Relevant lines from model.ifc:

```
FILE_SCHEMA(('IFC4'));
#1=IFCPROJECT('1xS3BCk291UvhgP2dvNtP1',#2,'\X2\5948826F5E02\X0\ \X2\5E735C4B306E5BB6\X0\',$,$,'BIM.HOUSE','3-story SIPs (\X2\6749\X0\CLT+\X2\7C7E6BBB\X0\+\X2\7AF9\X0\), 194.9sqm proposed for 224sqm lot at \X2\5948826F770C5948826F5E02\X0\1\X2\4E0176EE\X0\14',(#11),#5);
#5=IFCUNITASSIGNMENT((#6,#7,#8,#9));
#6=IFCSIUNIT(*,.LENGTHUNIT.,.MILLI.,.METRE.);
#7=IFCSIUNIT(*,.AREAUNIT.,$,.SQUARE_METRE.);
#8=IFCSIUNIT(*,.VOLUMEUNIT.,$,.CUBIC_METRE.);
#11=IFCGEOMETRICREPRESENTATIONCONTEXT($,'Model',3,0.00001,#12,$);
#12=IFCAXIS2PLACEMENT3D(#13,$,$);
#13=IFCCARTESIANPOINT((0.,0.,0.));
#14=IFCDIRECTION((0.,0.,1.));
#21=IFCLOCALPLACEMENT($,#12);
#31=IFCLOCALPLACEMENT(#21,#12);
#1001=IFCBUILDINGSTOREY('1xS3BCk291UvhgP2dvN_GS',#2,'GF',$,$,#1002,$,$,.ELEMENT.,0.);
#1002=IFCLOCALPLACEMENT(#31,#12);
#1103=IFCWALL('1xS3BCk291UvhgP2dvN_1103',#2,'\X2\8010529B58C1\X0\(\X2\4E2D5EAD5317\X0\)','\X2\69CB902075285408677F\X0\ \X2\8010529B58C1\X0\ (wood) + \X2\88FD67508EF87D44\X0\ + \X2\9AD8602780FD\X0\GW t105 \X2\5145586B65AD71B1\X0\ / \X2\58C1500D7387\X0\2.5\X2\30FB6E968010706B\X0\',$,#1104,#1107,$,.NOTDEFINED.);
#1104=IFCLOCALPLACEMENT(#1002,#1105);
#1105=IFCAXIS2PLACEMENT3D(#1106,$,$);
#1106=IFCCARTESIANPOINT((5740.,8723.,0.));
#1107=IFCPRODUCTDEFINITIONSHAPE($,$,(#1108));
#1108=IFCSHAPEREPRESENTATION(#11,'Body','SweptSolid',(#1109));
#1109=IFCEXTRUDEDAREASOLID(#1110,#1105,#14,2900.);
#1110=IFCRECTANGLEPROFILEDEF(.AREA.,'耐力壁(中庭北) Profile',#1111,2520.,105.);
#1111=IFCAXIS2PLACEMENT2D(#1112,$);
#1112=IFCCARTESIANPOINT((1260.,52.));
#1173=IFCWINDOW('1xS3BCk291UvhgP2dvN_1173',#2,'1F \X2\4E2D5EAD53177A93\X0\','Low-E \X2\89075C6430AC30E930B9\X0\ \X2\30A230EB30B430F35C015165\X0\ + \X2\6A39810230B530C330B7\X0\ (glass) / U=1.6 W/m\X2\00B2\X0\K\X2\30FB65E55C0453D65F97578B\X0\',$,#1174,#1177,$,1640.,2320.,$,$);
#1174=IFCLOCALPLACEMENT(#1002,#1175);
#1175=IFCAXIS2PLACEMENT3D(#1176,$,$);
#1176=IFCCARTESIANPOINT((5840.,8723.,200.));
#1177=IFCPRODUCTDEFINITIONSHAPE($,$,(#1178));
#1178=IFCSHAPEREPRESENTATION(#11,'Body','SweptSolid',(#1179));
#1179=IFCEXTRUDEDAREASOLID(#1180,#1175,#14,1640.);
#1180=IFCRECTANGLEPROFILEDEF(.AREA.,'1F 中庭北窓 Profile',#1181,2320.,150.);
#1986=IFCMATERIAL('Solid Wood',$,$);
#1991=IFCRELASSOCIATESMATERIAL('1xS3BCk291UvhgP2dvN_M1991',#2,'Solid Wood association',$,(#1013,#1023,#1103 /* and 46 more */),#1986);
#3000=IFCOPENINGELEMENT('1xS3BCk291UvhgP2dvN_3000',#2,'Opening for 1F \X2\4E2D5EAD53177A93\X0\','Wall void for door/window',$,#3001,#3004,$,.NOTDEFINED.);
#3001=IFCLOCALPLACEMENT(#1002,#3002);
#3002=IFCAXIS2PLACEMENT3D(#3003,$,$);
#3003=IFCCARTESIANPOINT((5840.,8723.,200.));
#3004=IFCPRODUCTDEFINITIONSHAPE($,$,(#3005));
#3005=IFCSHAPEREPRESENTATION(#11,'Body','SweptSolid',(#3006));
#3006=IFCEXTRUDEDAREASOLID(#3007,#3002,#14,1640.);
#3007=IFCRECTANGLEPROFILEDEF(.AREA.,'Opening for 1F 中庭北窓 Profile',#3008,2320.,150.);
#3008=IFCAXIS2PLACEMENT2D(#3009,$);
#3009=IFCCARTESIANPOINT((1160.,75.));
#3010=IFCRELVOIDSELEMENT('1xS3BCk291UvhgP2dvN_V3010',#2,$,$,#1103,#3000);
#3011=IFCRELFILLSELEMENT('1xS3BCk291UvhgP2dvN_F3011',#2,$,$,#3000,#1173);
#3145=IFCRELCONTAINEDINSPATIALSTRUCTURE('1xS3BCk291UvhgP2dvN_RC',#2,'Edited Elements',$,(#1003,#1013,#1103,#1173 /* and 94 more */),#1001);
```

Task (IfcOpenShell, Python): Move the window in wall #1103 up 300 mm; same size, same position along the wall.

```python
import numpy as np
import ifcopenshell
import ifcopenshell.api.geometry
import ifcopenshell.util.placement
import ifcopenshell.util.unit

model = ifcopenshell.open("model.ifc")
unit_scale = ifcopenshell.util.unit.calculate_unit_scale(model)

window = model.by_guid("1xS3BCk291UvhgP2dvN_1173")
opening = window.FillsVoids[0].RelatingOpeningElement
dz = 300.0

shift = np.array([0.0, 0.0, dz])
# The window is not placed relative to its opening, so move both.
for product in (opening, window):
    matrix = ifcopenshell.util.placement.get_local_placement(product.ObjectPlacement)
    matrix[:3, 3] += shift
    ifcopenshell.api.geometry.edit_object_placement(model, product=product, matrix=matrix, is_si=False)

print(f"moved by {dz * unit_scale:+.3f} m")

model.write("model_rev.ifc")
```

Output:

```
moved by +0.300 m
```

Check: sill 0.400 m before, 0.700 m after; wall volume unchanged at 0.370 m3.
